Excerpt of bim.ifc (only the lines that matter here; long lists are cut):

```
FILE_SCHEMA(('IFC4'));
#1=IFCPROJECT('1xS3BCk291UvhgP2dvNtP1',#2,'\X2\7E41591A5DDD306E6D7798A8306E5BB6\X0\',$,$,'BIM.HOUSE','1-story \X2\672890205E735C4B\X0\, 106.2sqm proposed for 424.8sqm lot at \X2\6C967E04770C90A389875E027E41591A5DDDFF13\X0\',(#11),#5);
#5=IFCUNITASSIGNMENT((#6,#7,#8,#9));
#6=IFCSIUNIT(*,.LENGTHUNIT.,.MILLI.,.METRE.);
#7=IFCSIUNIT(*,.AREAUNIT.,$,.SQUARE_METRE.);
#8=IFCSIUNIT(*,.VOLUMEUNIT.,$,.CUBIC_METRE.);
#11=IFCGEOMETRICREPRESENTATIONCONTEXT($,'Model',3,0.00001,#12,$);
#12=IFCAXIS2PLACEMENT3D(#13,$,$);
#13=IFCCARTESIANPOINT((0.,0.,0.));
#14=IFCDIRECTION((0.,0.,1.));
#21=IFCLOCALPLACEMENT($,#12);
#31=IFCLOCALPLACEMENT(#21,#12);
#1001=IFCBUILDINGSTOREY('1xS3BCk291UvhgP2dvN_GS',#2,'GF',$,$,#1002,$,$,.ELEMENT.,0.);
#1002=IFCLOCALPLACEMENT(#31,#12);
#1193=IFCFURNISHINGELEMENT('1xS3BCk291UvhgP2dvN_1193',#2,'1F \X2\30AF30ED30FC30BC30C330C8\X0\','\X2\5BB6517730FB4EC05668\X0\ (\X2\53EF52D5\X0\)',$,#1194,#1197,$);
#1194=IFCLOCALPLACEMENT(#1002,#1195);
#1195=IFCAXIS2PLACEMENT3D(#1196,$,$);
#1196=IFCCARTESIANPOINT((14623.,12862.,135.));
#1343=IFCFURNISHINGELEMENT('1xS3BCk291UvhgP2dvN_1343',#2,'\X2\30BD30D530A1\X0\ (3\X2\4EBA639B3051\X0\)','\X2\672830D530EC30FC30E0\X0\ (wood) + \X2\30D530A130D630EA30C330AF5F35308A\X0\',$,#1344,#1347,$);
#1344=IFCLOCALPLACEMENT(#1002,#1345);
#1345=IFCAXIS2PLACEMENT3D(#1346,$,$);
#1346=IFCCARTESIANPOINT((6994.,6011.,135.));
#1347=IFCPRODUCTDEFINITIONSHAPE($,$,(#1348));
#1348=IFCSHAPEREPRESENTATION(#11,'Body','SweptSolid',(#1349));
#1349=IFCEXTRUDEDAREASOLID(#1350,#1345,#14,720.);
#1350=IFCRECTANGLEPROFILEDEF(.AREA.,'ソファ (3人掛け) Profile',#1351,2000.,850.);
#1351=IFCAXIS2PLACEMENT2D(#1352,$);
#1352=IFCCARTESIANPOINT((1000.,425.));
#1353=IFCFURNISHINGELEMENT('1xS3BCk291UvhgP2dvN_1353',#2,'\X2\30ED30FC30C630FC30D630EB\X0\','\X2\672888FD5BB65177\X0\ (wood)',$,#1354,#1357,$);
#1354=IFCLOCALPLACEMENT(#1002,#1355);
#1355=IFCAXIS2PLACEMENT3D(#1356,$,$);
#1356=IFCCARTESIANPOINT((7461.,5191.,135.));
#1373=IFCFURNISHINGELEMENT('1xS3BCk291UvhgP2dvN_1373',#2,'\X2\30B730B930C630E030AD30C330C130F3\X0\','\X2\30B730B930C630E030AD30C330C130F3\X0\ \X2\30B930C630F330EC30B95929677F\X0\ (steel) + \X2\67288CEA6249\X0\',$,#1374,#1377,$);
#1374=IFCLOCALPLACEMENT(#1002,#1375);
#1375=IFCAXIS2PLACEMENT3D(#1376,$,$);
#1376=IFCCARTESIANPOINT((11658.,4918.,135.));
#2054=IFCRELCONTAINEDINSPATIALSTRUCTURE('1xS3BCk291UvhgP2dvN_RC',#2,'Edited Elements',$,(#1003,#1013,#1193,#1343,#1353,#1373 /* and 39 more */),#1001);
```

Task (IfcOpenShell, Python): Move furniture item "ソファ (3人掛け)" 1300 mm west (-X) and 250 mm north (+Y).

```python
import ifcopenshell
import ifcopenshell.api.geometry
import ifcopenshell.util.placement
import ifcopenshell.util.unit

model = ifcopenshell.open("bim.ifc")
unit_scale = ifcopenshell.util.unit.calculate_unit_scale(model)

item = model.by_id(1343)
matrix = ifcopenshell.util.placement.get_local_placement(item.ObjectPlacement)
matrix[0, 3] -= 1.3 / unit_scale
matrix[1, 3] += 0.25 / unit_scale
ifcopenshell.api.geometry.edit_object_placement(model, product=item, matrix=matrix, is_si=False)

print(ifcopenshell.util.placement.get_local_placement(item.ObjectPlacement).round(3) + 0.0)

model.write("bim_edited.ifc")
```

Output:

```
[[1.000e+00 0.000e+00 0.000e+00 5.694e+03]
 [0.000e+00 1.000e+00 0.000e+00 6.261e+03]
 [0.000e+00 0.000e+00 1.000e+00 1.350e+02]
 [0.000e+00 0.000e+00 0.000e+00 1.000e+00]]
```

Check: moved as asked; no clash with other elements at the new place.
